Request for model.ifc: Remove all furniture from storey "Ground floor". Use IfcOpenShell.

First a look at what the model holds.

```python
import ifcopenshell
import ifcopenshell.util.element

model = ifcopenshell.open("model.ifc")
print(model.schema)
storey = next(s for s in model.by_type("IfcBuildingStorey") if s.Name == "Ground floor")
furniture = [e for e in ifcopenshell.util.element.get_decomposition(storey) if e.is_a("IfcFurnishingElement")]
seen = {}
for e in furniture:
    element_type = ifcopenshell.util.element.get_type(e)
    name = element_type.Name if element_type not in (None, e) else None
    seen[name] = seen.get(name, 0) + 1
for name, count in sorted(seen.items(), key=str):
    print(count, "x", name)
```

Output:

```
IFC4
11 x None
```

```python
import ifcopenshell
import ifcopenshell.api.root
import ifcopenshell.util.element

model = ifcopenshell.open("model.ifc")

storey = next(s for s in model.by_type("IfcBuildingStorey") if s.Name == "Ground floor")
furniture = [e for e in ifcopenshell.util.element.get_decomposition(storey) if e.is_a("IfcFurnishingElement")]

for e in furniture:
    ifcopenshell.api.root.remove_product(model, product=e)
print(len(furniture), "removed")

model.write("model-out.ifc")
```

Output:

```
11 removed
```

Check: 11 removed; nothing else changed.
